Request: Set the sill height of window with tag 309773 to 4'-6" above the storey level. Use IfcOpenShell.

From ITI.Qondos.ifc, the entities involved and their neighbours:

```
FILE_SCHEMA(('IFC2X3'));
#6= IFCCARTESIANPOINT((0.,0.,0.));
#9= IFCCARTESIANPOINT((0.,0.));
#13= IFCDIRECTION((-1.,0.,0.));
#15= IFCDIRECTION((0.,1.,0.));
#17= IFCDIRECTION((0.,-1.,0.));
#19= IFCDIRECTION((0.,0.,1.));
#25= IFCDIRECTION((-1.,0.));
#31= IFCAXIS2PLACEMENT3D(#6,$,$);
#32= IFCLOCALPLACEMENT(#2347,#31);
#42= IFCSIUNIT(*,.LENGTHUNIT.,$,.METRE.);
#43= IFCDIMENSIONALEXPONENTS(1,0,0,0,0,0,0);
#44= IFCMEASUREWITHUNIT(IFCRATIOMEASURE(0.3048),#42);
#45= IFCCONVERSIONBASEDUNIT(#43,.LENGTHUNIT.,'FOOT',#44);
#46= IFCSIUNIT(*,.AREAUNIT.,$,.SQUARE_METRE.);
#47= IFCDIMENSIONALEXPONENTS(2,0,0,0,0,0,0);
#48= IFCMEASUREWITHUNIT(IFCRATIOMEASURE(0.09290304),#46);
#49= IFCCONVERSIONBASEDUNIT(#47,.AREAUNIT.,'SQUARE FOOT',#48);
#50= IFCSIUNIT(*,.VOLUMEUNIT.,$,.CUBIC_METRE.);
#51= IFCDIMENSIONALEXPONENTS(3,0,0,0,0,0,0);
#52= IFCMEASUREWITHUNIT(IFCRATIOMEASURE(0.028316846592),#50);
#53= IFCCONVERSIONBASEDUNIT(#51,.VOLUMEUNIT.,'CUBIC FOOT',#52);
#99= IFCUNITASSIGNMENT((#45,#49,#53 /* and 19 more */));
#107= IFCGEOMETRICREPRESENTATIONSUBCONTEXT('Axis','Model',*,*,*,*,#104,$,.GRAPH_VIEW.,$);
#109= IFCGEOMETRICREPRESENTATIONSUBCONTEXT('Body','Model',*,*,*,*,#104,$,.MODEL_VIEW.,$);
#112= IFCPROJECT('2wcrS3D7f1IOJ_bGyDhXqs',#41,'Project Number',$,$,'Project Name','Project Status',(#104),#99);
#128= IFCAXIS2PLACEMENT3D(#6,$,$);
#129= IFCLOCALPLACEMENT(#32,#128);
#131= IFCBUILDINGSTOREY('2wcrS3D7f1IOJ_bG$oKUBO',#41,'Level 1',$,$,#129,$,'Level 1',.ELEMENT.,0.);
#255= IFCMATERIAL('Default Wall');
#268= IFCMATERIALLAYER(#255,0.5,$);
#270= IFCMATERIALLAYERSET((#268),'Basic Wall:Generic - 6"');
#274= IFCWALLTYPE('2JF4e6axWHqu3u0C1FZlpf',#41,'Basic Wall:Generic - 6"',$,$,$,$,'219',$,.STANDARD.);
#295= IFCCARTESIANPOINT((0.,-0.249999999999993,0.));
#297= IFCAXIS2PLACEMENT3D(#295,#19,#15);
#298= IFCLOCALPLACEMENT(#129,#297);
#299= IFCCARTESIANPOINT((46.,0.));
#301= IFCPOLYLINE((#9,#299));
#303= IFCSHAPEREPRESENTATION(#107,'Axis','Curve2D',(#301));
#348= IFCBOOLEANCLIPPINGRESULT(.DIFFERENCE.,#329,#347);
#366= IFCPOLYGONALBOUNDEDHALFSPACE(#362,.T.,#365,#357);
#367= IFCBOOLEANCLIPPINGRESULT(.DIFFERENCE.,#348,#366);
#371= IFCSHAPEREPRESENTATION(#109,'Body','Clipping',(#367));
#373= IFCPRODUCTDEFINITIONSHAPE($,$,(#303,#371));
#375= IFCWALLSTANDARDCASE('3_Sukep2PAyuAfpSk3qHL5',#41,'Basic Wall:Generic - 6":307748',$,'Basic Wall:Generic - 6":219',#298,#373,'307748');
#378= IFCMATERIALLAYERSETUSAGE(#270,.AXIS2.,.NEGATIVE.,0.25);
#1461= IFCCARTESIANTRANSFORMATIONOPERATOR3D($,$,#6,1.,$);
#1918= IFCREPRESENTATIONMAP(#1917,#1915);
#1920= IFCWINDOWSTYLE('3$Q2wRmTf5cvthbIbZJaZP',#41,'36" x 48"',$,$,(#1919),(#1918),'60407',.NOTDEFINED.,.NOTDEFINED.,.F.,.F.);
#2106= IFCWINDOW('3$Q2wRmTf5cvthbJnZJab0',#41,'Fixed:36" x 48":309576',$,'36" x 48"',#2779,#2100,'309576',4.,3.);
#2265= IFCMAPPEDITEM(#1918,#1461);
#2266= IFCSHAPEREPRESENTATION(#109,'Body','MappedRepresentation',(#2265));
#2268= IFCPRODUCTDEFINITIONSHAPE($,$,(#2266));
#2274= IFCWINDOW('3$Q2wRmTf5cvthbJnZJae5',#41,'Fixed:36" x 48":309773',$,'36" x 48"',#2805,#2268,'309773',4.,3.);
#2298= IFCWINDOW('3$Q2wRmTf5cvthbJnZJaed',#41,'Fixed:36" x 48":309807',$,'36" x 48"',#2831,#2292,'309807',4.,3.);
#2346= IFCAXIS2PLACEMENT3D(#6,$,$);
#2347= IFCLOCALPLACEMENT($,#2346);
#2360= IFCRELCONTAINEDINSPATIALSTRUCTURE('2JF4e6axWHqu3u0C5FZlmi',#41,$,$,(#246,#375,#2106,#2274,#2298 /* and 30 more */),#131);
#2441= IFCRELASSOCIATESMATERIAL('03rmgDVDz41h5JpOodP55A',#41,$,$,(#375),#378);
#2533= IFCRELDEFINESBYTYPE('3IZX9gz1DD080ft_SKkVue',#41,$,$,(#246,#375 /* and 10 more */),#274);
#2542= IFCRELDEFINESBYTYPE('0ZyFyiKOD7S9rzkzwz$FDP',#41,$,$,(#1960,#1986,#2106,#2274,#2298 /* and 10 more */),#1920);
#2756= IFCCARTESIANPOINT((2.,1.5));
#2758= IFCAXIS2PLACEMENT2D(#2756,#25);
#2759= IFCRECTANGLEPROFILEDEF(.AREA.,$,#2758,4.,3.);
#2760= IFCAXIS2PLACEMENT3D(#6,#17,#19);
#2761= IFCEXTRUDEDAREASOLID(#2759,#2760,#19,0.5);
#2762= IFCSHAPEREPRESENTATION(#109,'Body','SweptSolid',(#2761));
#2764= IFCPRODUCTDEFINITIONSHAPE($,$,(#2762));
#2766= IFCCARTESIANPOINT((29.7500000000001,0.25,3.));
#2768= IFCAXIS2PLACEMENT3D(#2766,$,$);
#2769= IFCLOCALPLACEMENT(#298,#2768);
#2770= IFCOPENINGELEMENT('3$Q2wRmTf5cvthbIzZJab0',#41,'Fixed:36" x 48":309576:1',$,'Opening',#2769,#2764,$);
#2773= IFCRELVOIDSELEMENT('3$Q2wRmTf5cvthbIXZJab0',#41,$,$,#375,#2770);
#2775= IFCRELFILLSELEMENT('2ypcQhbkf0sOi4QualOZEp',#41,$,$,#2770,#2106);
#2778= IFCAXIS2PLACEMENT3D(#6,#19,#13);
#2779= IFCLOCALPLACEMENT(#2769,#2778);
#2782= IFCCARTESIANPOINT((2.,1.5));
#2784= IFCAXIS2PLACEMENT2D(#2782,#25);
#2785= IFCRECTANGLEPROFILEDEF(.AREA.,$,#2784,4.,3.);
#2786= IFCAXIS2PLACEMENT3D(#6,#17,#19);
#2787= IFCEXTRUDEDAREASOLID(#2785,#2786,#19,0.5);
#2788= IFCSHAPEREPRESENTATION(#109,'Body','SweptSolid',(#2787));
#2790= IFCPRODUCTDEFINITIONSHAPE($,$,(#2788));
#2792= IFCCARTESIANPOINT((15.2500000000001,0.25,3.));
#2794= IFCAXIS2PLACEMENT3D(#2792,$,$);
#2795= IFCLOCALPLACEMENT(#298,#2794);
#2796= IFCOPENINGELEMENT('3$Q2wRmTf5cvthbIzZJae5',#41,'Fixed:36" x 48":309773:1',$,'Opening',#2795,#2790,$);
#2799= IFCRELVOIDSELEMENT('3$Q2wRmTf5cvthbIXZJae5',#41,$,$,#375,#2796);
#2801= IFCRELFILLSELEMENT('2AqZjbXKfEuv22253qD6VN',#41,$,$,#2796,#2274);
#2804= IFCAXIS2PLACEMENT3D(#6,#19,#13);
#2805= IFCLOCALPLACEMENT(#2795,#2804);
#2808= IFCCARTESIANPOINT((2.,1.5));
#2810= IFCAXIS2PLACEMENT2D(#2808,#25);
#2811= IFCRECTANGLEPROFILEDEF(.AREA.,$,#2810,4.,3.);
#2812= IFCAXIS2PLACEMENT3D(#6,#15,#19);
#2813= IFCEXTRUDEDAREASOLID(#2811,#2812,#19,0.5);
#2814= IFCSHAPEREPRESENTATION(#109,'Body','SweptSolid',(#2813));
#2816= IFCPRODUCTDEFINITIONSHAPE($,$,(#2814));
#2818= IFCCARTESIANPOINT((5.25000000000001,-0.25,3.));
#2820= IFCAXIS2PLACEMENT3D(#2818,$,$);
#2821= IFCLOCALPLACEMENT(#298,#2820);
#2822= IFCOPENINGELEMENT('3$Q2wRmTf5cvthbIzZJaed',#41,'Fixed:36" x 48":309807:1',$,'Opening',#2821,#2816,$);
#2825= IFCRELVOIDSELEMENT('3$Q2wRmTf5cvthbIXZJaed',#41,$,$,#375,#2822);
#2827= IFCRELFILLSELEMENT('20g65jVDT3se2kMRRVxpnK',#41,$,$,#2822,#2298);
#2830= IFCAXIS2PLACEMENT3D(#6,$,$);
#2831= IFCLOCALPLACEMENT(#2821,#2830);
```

```python
import numpy as np
import ifcopenshell
import ifcopenshell.api.geometry
import ifcopenshell.geom
import ifcopenshell.util.element
import ifcopenshell.util.placement
import ifcopenshell.util.shape
import ifcopenshell.util.unit

model = ifcopenshell.open("ITI.Qondos.ifc")
unit_scale = ifcopenshell.util.unit.calculate_unit_scale(model)

window = model.by_guid("3$Q2wRmTf5cvthbJnZJae5")
opening = window.FillsVoids[0].RelatingOpeningElement
storey = ifcopenshell.util.element.get_container(window, ifc_class="IfcBuildingStorey")
level = ifcopenshell.util.placement.get_local_placement(storey.ObjectPlacement)[2, 3]

# The opening's origin need not be at the sill, so measure its lowest point.
shape = ifcopenshell.geom.create_shape(ifcopenshell.geom.settings(), opening)
bottom = ifcopenshell.util.shape.get_shape_bottom_elevation(shape, shape.geometry) / unit_scale
dz = level + 54 * 0.0254 / unit_scale - bottom

shift = np.array([0.0, 0.0, dz])
# The window is placed relative to its opening, so it follows when the opening moves.
matrix = ifcopenshell.util.placement.get_local_placement(opening.ObjectPlacement)
matrix[:3, 3] += shift
ifcopenshell.api.geometry.edit_object_placement(
    model, product=opening, matrix=matrix, is_si=False, should_transform_children=True
)

print(f"moved by {dz * unit_scale:+.3f} m")

model.write("ITI.Qondos_updated.ifc")
```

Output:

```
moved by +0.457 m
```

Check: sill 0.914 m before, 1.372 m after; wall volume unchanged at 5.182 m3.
